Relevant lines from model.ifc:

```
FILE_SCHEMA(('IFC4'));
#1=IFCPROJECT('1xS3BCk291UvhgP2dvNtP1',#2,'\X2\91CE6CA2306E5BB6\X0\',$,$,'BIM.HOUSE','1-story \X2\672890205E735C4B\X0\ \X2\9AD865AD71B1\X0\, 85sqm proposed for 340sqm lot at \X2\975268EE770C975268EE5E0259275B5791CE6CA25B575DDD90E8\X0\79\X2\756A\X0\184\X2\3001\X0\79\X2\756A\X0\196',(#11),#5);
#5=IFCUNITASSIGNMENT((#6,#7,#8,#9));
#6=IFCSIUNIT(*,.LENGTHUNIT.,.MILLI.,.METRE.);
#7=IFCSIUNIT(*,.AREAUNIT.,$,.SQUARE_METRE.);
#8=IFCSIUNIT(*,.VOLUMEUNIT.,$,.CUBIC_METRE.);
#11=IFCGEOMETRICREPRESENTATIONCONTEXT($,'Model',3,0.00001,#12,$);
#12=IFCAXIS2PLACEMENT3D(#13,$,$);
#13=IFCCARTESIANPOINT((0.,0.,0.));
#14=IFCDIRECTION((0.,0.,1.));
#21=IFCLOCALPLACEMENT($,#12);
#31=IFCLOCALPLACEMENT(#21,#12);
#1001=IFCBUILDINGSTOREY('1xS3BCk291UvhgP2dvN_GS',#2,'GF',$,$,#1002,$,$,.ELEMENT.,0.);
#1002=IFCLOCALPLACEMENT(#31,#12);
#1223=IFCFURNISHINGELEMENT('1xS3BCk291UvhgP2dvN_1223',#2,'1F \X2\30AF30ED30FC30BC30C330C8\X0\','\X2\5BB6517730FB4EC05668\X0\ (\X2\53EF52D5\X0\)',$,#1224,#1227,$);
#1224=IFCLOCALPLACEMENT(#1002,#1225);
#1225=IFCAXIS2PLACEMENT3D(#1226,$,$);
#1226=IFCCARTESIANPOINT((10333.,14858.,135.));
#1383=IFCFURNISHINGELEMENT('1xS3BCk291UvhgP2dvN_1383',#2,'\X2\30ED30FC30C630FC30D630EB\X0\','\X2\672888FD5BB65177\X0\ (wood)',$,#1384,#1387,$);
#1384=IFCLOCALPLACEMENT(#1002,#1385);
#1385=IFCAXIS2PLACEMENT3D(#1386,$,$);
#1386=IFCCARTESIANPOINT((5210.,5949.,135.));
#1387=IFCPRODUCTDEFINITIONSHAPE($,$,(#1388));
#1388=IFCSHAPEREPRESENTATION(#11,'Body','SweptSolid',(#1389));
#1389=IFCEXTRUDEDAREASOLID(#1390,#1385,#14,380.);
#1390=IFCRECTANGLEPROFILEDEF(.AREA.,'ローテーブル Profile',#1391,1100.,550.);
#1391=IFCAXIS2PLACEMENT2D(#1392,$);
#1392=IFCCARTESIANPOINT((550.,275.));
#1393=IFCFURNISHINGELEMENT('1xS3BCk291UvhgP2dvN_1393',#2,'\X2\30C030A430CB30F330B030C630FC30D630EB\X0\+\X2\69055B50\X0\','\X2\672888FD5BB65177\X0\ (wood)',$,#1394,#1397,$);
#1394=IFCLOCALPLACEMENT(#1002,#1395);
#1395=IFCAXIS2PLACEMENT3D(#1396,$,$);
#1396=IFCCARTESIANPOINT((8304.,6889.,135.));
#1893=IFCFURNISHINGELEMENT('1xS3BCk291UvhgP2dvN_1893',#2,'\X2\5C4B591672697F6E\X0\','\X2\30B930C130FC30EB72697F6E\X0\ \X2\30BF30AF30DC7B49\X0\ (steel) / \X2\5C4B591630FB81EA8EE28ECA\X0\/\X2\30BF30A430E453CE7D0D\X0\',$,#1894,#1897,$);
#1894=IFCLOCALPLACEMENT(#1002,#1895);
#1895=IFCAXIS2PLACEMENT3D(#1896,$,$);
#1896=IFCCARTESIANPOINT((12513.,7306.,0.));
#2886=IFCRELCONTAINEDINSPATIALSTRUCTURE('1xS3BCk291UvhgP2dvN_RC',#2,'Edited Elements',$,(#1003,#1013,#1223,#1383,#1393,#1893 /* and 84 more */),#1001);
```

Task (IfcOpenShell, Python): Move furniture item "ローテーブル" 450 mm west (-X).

```python
import ifcopenshell
import ifcopenshell.api.geometry
import ifcopenshell.util.placement

model = ifcopenshell.open("model.ifc")

item = model.by_guid("1xS3BCk291UvhgP2dvN_1383")
matrix = ifcopenshell.util.placement.get_local_placement(item.ObjectPlacement)
matrix[0, 3] -= 450.0
ifcopenshell.api.geometry.edit_object_placement(model, product=item, matrix=matrix, is_si=False)

print(ifcopenshell.util.placement.get_local_placement(item.ObjectPlacement).round(3) + 0.0)

model.write("model_edited.ifc")
```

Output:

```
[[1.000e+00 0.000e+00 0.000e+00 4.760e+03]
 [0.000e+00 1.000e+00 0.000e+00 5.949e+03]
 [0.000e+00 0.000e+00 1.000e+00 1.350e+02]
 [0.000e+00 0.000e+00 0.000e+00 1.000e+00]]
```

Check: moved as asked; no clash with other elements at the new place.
